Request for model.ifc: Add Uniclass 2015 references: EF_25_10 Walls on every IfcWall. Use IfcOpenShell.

First a look at what the model holds.

```python
import ifcopenshell

model = ifcopenshell.open("model.ifc")
print(model.schema)
print("classifications:", [c.Name for c in model.by_type("IfcClassification")])
for ifc_class in ("IfcDoor", "IfcRoof", "IfcStair", "IfcWall", "IfcWindow"):
    print(ifc_class, len(model.by_type(ifc_class)))
```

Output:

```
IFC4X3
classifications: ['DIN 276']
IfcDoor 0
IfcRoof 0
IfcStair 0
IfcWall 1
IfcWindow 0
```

```python
import ifcopenshell
import ifcopenshell.api.classification

model = ifcopenshell.open("model.ifc")

system = ifcopenshell.api.classification.add_classification(model, classification="Uniclass 2015")

codes = {
    "IfcWall": ("EF_25_10", "Walls"),
}
for ifc_class, (code, name) in codes.items():
    products = model.by_type(ifc_class)
    ifcopenshell.api.classification.add_reference(
        model, products=products, classification=system, identification=code, name=name
    )
    print(code, len(products))

model.write("model_rev.ifc")
```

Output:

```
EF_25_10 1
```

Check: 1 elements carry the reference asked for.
